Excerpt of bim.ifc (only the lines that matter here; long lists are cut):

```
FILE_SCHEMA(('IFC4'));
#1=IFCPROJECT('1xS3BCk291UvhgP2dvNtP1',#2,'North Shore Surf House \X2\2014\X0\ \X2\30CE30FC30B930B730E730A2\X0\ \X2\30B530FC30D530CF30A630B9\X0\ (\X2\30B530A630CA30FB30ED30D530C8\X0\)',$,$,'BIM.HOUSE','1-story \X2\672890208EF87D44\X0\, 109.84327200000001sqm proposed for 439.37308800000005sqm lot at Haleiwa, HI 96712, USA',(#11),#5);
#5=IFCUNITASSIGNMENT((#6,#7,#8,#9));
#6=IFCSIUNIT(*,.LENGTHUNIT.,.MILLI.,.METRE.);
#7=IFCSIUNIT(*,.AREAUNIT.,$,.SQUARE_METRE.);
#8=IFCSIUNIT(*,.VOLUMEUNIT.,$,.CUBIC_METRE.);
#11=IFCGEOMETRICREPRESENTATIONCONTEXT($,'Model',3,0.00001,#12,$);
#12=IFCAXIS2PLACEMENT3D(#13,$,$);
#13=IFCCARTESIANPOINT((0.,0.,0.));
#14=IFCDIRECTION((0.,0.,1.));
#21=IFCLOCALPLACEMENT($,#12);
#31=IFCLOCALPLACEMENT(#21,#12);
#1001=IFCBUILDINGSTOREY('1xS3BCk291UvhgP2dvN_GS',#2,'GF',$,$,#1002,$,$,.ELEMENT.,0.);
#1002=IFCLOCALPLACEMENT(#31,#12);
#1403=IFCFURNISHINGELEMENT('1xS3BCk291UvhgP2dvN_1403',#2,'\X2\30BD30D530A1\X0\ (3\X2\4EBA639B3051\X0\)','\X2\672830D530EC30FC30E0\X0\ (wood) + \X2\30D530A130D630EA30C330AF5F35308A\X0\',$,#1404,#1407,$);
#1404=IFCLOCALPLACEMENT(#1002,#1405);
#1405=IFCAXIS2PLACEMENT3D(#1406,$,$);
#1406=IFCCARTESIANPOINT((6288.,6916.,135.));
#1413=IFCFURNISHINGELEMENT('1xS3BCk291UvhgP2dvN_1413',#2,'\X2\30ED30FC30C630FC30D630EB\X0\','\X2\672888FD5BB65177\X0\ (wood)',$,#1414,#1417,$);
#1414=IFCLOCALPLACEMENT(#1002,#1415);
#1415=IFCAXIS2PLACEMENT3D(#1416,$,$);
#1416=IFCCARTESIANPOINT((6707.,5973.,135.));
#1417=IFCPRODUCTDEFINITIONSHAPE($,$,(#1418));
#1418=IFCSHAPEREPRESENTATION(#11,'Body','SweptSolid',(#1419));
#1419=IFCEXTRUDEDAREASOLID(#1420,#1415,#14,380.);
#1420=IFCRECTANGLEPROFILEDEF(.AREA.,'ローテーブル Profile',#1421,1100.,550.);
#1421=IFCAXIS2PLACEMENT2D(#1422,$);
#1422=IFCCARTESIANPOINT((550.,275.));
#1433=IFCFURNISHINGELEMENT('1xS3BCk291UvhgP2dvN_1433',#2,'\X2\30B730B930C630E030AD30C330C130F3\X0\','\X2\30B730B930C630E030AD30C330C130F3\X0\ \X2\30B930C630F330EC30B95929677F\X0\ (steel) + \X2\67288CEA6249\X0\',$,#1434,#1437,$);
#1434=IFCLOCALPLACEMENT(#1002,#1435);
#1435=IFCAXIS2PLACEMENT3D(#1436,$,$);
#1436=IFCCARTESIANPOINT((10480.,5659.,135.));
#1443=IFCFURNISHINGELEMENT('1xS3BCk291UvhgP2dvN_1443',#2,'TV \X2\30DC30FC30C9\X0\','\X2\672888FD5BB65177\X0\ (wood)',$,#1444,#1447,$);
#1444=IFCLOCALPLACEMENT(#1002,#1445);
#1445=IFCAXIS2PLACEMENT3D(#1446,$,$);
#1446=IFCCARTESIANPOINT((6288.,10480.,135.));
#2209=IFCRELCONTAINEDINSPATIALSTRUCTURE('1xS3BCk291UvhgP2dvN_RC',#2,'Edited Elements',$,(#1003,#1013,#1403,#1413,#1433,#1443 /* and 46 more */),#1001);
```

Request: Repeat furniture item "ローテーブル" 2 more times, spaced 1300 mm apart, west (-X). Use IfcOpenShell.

```python
import numpy as np
import ifcopenshell
import ifcopenshell.api.geometry
import ifcopenshell.api.root
import ifcopenshell.util.element
import ifcopenshell.util.placement
import ifcopenshell.util.unit

model = ifcopenshell.open("bim.ifc")
unit_scale = ifcopenshell.util.unit.calculate_unit_scale(model)


def reuse_history(source, copy):
    """copy_class also copies each property set's owner history, people and application; keep the originals."""
    for rel in copy.IsDefinedBy:
        if rel.is_a("IfcRelDefinesByProperties") and (history := rel.RelatingPropertyDefinition.OwnerHistory):
            rel.RelatingPropertyDefinition.OwnerHistory = source.OwnerHistory
            ifcopenshell.util.element.remove_deep2(model, history)


source = model.by_id(1413)
base = ifcopenshell.util.placement.get_local_placement(source.ObjectPlacement)
step = np.array([-1.0, 0.0, 0.0]) * 1.3 / unit_scale

for i in range(1, 3):
    copy = ifcopenshell.api.root.copy_class(model, product=source)
    copy.Representation = ifcopenshell.util.element.copy_deep(
        model, source.Representation, exclude=["IfcGeometricRepresentationContext", "IfcRepresentationMap"]
    )
    reuse_history(source, copy)
    matrix = base.copy()
    matrix[:3, 3] += i * step
    print("added at", matrix[:3, 3].round(3) + 0.0)
    ifcopenshell.api.geometry.edit_object_placement(model, product=copy, matrix=matrix, is_si=False)

model.write("bim-out.ifc")
```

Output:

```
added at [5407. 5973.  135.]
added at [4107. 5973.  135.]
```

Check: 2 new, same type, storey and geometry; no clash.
